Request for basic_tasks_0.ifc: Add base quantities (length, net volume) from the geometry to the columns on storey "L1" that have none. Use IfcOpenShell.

First a look at what the model holds.

```python
import ifcopenshell
import ifcopenshell.util.element
import ifcopenshell.util.unit

model = ifcopenshell.open("basic_tasks_0.ifc")
print(model.schema)
for unit_type in ("LENGTHUNIT", "AREAUNIT", "VOLUMEUNIT"):
    print(unit_type, ifcopenshell.util.unit.calculate_unit_scale(model, unit_type))
storey = next(s for s in model.by_type("IfcBuildingStorey") if s.Name == "L1")
columns = [e for e in ifcopenshell.util.element.get_decomposition(storey) if e.is_a("IfcColumn")]
for e in sorted(columns, key=lambda e: e.id()):
    print(e.id(), e.is_a(), e.Name, list(ifcopenshell.util.element.get_psets(e, qtos_only=True)), sep=" | ")
```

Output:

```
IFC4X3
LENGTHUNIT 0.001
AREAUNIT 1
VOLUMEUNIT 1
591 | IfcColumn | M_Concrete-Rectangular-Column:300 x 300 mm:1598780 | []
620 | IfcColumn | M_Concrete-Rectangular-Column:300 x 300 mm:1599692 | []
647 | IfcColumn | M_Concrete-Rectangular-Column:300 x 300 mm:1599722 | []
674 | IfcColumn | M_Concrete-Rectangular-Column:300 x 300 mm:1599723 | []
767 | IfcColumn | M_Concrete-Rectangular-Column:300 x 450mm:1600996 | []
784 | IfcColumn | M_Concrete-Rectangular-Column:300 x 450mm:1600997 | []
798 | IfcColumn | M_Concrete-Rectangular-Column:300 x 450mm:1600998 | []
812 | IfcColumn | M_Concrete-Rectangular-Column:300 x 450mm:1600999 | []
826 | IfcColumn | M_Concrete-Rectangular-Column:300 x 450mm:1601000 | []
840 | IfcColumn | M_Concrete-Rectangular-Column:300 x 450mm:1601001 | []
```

```python
import ifcopenshell
import ifcopenshell.api.pset
import ifcopenshell.geom
import ifcopenshell.util.element
import ifcopenshell.util.shape
import ifcopenshell.util.unit

model = ifcopenshell.open("basic_tasks_0.ifc")
unit_scale = ifcopenshell.util.unit.calculate_unit_scale(model)
volume_scale = ifcopenshell.util.unit.calculate_unit_scale(model, "VOLUMEUNIT")
settings = ifcopenshell.geom.settings()

storey = next(s for s in model.by_type("IfcBuildingStorey") if s.Name == "L1")
columns = [e for e in ifcopenshell.util.element.get_decomposition(storey) if e.is_a("IfcColumn")]

for e in sorted(columns, key=lambda e: e.id()):
    if ifcopenshell.util.element.get_psets(e, qtos_only=True, should_inherit=False):
        continue
    # Geometry comes back in metres, in the element's own axes.
    shape = ifcopenshell.geom.create_shape(settings, e)
    values = {
        "Length": ifcopenshell.util.shape.get_z(shape.geometry) / unit_scale,
        "NetVolume": ifcopenshell.util.shape.get_volume(shape.geometry) / volume_scale,
    }
    qto = ifcopenshell.api.pset.add_qto(model, product=e, name="Qto_ColumnBaseQuantities")
    ifcopenshell.api.pset.edit_qto(model, qto=qto, properties=values)
    print(e.id(), {k: round(v, 3) for k, v in values.items()})

model.write("basic_tasks_0_edited.ifc")
```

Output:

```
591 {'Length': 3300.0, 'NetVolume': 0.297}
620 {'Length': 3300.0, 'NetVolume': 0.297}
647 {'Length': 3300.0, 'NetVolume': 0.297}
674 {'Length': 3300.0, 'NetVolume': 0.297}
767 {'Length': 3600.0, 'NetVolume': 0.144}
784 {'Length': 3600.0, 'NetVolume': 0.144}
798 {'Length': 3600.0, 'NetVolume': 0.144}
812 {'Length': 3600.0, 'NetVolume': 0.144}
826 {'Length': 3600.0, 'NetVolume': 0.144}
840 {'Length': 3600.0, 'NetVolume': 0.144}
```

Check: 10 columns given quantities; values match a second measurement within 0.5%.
